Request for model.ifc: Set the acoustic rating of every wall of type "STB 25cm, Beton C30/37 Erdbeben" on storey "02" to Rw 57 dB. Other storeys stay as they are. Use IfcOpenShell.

First a look at what the model holds.

```python
import ifcopenshell
import ifcopenshell.util.element

model = ifcopenshell.open("model.ifc")
print(model.schema)
storey = next(s for s in model.by_type("IfcBuildingStorey") if s.Name == "02")
walls = [e for e in ifcopenshell.util.element.get_decomposition(storey) if e.is_a("IfcWall")]
seen = {}
for e in walls:
    element_type = ifcopenshell.util.element.get_type(e)
    key = (element_type.Name if element_type != e and element_type else None, ifcopenshell.util.element.get_pset(e, "Pset_WallCommon", "AcousticRating"))
    seen[key] = seen.get(key, 0) + 1
for (name, value), count in sorted(seen.items(), key=str):
    print(count, "x", name, "|", value)
```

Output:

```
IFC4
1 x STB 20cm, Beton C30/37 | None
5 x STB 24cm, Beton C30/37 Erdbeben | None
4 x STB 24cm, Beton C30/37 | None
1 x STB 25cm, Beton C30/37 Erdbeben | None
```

```python
import ifcopenshell
import ifcopenshell.api.pset
import ifcopenshell.util.element

model = ifcopenshell.open("model.ifc")

storey = next(s for s in model.by_type("IfcBuildingStorey") if s.Name == "02")
walls = [e for e in ifcopenshell.util.element.get_decomposition(storey) if e.is_a("IfcWall")]

count = 0
for e in walls:
    element_type = ifcopenshell.util.element.get_type(e)
    if element_type in (None, e) or element_type.Name != "STB 25cm, Beton C30/37 Erdbeben":
        continue
    # add_pset returns the element's existing set when there is one.
    pset = ifcopenshell.api.pset.add_pset(model, product=e, name="Pset_WallCommon")
    ifcopenshell.api.pset.edit_pset(model, pset=pset, properties={"AcousticRating": "Rw 57 dB"})
    count += 1

print(count, "walls updated")

model.write("model-out.ifc")
```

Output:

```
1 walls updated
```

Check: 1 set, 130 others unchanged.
